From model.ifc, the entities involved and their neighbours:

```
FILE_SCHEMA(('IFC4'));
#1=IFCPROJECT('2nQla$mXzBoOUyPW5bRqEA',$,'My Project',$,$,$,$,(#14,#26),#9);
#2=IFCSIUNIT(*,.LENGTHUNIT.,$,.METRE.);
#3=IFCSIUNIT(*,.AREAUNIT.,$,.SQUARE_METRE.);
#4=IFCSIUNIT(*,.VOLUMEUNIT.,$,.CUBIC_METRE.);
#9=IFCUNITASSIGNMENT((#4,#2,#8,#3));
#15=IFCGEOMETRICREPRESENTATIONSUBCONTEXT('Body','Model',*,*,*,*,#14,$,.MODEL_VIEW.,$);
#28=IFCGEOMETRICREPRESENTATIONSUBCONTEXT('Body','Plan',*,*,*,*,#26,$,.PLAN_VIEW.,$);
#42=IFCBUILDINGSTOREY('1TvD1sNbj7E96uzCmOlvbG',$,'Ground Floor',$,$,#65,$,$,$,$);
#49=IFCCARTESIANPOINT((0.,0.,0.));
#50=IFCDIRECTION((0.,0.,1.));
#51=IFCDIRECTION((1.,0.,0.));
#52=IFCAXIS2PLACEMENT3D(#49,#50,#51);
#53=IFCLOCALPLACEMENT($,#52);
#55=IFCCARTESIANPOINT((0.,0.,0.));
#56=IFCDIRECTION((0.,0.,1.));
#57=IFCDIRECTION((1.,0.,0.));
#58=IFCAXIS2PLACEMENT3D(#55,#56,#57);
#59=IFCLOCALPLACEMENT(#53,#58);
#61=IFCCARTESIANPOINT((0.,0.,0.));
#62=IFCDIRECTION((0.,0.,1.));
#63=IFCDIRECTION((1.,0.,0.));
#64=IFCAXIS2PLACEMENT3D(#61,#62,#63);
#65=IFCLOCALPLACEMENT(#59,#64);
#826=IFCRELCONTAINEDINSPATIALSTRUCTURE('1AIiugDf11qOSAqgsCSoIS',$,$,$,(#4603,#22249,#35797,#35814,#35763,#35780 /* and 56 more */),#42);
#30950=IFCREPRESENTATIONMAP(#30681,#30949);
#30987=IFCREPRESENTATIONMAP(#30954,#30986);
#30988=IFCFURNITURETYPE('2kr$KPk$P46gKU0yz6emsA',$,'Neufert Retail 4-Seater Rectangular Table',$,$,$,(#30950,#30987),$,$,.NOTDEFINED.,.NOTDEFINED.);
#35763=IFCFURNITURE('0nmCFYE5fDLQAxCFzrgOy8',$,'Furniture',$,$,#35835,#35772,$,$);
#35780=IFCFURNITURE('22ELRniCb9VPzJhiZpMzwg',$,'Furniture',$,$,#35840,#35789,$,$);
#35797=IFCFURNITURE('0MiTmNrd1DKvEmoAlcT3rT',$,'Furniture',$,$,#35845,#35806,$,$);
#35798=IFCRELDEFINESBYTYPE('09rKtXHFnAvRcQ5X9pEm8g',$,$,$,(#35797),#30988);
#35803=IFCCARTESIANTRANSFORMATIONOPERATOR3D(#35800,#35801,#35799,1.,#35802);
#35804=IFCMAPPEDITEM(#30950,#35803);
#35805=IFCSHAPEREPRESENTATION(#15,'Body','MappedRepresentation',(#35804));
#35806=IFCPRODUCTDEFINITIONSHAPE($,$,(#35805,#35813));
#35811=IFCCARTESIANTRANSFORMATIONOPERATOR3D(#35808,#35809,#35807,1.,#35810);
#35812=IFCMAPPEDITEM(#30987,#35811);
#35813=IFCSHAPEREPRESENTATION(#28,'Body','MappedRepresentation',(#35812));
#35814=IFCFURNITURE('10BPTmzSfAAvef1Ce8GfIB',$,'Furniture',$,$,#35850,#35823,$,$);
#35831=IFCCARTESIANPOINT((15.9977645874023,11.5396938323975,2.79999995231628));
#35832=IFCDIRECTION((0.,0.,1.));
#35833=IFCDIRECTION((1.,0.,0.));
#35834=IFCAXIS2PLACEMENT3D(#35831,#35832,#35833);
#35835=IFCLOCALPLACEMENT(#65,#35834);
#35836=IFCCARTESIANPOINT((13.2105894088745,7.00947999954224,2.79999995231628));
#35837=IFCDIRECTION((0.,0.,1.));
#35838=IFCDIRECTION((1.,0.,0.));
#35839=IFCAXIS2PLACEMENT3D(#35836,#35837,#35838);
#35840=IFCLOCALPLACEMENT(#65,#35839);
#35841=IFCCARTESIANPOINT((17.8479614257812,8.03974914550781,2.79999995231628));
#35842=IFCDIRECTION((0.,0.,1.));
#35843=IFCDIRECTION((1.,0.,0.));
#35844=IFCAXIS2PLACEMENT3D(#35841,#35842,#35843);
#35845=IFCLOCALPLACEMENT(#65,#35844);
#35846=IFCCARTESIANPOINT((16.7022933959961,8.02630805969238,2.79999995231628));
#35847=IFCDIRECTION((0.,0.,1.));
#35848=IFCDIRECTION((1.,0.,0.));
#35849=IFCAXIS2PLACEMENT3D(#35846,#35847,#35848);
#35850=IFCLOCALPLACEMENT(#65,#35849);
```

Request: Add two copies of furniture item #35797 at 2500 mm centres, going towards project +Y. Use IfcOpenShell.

```python
import numpy as np
import ifcopenshell
import ifcopenshell.api.geometry
import ifcopenshell.api.root
import ifcopenshell.util.element
import ifcopenshell.util.placement

model = ifcopenshell.open("model.ifc")

source = model.by_guid("0MiTmNrd1DKvEmoAlcT3rT")
base = ifcopenshell.util.placement.get_local_placement(source.ObjectPlacement)
step = np.array([0.0, 1.0, 0.0]) * 2.5

for i in range(1, 3):
    copy = ifcopenshell.api.root.copy_class(model, product=source)
    copy.Representation = ifcopenshell.util.element.copy_deep(
        model, source.Representation, exclude=["IfcGeometricRepresentationContext", "IfcRepresentationMap"]
    )
    matrix = base.copy()
    matrix[:3, 3] += i * step
    print("added at", matrix[:3, 3].round(3) + 0.0)
    ifcopenshell.api.geometry.edit_object_placement(model, product=copy, matrix=matrix, is_si=False)

model.write("model_v2.ifc")
```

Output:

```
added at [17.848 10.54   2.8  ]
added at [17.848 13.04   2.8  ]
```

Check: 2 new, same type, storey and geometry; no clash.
